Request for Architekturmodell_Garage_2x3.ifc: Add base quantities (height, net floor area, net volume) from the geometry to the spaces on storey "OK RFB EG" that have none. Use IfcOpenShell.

First a look at what the model holds.

```python
import ifcopenshell
import ifcopenshell.util.element
import ifcopenshell.util.unit

model = ifcopenshell.open("Architekturmodell_Garage_2x3.ifc")
print(model.schema)
for unit_type in ("LENGTHUNIT", "AREAUNIT", "VOLUMEUNIT"):
    print(unit_type, ifcopenshell.util.unit.calculate_unit_scale(model, unit_type))
storey = next(s for s in model.by_type("IfcBuildingStorey") if s.Name == "OK RFB EG")
spaces = [e for e in ifcopenshell.util.element.get_decomposition(storey) if e.is_a("IfcSpace")]
for e in sorted(spaces, key=lambda e: e.id()):
    print(e.id(), e.is_a(), e.Name, list(ifcopenshell.util.element.get_psets(e, qtos_only=True)), sep=" | ")
```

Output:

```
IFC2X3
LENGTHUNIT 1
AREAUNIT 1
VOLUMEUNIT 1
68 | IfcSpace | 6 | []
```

```python
import ifcopenshell
import ifcopenshell.api.pset
import ifcopenshell.geom
import ifcopenshell.util.element
import ifcopenshell.util.shape
import ifcopenshell.util.unit

model = ifcopenshell.open("Architekturmodell_Garage_2x3.ifc")
unit_scale = ifcopenshell.util.unit.calculate_unit_scale(model)
area_scale = ifcopenshell.util.unit.calculate_unit_scale(model, "AREAUNIT")
volume_scale = ifcopenshell.util.unit.calculate_unit_scale(model, "VOLUMEUNIT")
settings = ifcopenshell.geom.settings()

storey = next(s for s in model.by_type("IfcBuildingStorey") if s.Name == "OK RFB EG")
spaces = [e for e in ifcopenshell.util.element.get_decomposition(storey) if e.is_a("IfcSpace")]

for e in sorted(spaces, key=lambda e: e.id()):
    if ifcopenshell.util.element.get_psets(e, qtos_only=True, should_inherit=False):
        continue
    # Geometry comes back in metres, in the element's own axes.
    shape = ifcopenshell.geom.create_shape(settings, e)
    values = {
        "Height": ifcopenshell.util.shape.get_z(shape.geometry) / unit_scale,
        "NetFloorArea": ifcopenshell.util.shape.get_footprint_area(shape.geometry) / area_scale,
        "NetVolume": ifcopenshell.util.shape.get_volume(shape.geometry) / volume_scale,
    }
    qto = ifcopenshell.api.pset.add_qto(model, product=e, name="BaseQuantities")
    ifcopenshell.api.pset.edit_qto(model, qto=qto, properties=values)
    print(e.id(), {k: round(v, 3) for k, v in values.items()})

model.write("Architekturmodell_Garage_2x3_edited.ifc")
```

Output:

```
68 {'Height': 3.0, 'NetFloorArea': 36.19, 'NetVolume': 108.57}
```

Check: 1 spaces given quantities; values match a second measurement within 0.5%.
